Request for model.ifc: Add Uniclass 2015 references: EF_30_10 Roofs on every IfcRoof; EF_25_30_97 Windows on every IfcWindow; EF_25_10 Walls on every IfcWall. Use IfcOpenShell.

First a look at what the model holds.

```python
import ifcopenshell

model = ifcopenshell.open("model.ifc")
print(model.schema)
print("classifications:", [c.Name for c in model.by_type("IfcClassification")])
for ifc_class in ("IfcDoor", "IfcRoof", "IfcStair", "IfcWall", "IfcWindow"):
    print(ifc_class, len(model.by_type(ifc_class)))
```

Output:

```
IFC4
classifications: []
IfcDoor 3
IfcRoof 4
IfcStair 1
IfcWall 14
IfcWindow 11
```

```python
import ifcopenshell
import ifcopenshell.api.classification

model = ifcopenshell.open("model.ifc")

system = ifcopenshell.api.classification.add_classification(model, classification="Uniclass 2015")

codes = {
    "IfcRoof": ("EF_30_10", "Roofs"),
    "IfcWindow": ("EF_25_30_97", "Windows"),
    "IfcWall": ("EF_25_10", "Walls"),
}
for ifc_class, (code, name) in codes.items():
    products = model.by_type(ifc_class)
    ifcopenshell.api.classification.add_reference(
        model, products=products, classification=system, identification=code, name=name
    )
    print(code, len(products))

model.write("model_v2.ifc")
```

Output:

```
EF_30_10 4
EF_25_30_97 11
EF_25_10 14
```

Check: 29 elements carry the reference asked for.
